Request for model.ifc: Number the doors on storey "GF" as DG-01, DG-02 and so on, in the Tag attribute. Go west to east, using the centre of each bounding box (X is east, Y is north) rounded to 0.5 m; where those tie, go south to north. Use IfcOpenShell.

First a look at what the model holds.

```python
import ifcopenshell
import ifcopenshell.util.element
import ifcopenshell.util.placement

model = ifcopenshell.open("model.ifc")
print(model.schema)
storey = next(s for s in model.by_type("IfcBuildingStorey") if s.Name == "GF")
doors = [e for e in ifcopenshell.util.element.get_decomposition(storey) if e.is_a("IfcDoor")]
for e in sorted(doors, key=lambda e: e.id()):
    origin = ifcopenshell.util.placement.get_local_placement(e.ObjectPlacement)[:3, 3]
    print(e.id(), e.Tag, e.Name, origin.round(2) + 0.0, sep=" | ")
```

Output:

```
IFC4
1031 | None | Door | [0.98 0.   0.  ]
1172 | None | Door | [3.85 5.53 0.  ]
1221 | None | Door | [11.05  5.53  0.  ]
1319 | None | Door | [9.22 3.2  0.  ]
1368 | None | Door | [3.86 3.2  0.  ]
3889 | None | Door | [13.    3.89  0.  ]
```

```python
import ifcopenshell
import ifcopenshell.geom
import ifcopenshell.util.element
import ifcopenshell.util.shape

model = ifcopenshell.open("model.ifc")
settings = ifcopenshell.geom.settings()
settings.set("use-world-coords", True)


def centre(element):
    shape = ifcopenshell.geom.create_shape(settings, element)
    return ifcopenshell.util.shape.get_bbox_centroid(shape.geometry)


storey = next(s for s in model.by_type("IfcBuildingStorey") if s.Name == "GF")
doors = [e for e in ifcopenshell.util.element.get_decomposition(storey) if e.is_a("IfcDoor")]

# Insertion points can sit at a corner or the storey origin, so sort by the geometry (in metres).
centres = {e: centre(e) for e in doors}
doors.sort(key=lambda e: (round(centres[e][0] / 0.5), centres[e][1]))

for i, e in enumerate(doors, start=1):
    number = f"DG-{i:02d}"
    e.Tag = number
    print(e.id(), number)

model.write("model-out.ifc")
```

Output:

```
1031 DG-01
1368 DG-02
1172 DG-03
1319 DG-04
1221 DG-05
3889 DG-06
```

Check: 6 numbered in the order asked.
